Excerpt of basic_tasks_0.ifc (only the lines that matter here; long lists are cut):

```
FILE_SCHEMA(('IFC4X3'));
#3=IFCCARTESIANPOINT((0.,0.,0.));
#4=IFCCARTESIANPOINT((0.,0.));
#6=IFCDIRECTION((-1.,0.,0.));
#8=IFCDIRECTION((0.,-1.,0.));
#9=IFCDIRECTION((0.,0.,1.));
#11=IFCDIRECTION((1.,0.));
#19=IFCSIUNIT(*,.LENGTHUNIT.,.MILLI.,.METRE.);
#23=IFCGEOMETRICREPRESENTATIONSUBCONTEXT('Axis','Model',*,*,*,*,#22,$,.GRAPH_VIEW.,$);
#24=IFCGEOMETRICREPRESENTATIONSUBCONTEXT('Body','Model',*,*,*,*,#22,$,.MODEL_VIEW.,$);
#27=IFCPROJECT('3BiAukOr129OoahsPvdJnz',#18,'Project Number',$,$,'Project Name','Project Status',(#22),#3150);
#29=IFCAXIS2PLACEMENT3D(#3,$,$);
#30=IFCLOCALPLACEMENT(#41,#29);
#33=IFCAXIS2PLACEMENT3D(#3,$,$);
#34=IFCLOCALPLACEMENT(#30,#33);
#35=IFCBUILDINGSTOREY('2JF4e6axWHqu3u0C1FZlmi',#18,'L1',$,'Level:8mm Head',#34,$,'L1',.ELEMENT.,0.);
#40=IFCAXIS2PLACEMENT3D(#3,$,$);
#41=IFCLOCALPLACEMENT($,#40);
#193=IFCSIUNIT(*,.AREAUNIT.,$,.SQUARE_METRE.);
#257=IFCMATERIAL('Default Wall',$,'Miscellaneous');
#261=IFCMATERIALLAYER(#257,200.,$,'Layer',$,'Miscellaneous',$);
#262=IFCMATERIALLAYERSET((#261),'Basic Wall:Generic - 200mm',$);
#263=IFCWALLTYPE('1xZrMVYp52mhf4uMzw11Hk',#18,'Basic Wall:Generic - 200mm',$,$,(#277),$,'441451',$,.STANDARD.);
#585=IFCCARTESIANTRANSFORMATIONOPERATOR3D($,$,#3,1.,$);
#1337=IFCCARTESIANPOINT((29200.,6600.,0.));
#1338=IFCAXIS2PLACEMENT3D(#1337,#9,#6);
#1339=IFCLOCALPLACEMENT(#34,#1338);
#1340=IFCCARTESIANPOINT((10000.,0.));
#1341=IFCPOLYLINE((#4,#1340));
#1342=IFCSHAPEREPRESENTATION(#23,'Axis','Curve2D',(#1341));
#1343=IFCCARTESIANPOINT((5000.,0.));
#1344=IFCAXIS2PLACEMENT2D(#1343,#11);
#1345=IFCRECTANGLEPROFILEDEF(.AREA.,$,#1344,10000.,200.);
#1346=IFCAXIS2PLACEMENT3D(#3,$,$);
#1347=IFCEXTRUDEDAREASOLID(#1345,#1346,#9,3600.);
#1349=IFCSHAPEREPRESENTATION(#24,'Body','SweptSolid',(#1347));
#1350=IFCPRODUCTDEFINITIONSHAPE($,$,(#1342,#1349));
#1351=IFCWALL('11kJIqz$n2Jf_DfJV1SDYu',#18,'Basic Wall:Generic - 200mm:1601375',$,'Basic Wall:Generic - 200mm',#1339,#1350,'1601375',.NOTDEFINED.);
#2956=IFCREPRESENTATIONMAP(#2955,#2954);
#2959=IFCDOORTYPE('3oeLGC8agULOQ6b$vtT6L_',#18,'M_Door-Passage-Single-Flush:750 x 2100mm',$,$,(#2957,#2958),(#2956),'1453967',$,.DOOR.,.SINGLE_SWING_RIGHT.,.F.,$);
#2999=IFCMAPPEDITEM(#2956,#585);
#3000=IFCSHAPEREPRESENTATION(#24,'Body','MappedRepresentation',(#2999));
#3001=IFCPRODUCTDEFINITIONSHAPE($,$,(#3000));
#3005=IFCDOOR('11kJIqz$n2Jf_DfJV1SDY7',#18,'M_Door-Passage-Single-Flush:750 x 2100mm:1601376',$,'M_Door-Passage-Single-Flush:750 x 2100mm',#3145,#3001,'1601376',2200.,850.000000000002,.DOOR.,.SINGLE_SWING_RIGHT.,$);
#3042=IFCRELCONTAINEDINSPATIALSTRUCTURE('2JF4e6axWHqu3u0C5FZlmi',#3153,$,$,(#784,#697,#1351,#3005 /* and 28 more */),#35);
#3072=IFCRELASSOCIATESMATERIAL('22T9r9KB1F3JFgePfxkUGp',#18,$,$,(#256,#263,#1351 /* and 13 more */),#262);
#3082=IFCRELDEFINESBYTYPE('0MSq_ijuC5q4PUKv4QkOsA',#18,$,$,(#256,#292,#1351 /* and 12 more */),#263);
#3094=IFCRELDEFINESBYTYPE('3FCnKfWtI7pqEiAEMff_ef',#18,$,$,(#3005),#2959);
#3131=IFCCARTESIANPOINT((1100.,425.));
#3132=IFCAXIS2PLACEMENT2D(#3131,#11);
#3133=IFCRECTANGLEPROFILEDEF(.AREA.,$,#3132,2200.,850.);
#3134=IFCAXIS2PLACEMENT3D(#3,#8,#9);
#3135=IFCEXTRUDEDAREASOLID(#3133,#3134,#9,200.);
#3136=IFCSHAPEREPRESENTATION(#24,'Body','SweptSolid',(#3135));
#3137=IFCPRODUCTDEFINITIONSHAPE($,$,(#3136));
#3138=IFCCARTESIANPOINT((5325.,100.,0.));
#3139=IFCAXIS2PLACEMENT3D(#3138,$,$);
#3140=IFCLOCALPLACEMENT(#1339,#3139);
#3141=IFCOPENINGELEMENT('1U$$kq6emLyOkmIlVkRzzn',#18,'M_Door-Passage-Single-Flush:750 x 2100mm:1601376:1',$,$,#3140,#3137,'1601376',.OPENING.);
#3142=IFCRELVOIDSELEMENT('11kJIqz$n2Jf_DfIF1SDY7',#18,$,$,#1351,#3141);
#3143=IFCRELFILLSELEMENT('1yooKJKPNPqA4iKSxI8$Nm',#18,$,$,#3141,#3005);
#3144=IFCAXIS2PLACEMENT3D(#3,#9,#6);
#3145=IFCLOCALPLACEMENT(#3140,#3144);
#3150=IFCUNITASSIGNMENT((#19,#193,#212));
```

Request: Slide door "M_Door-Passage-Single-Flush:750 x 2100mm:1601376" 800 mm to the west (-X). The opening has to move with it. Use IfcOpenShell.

```python
import ifcopenshell
import ifcopenshell.api.geometry
import ifcopenshell.util.placement
import ifcopenshell.util.unit

model = ifcopenshell.open("basic_tasks_0.ifc")
unit_scale = ifcopenshell.util.unit.calculate_unit_scale(model)

door = model.by_id(3005)
opening = door.FillsVoids[0].RelatingOpeningElement
wall = opening.VoidsElements[0].RelatingBuildingElement

wall_matrix = ifcopenshell.util.placement.get_local_placement(wall.ObjectPlacement)
shift = wall_matrix[:3, 0] * 0.8 / unit_scale
before = ifcopenshell.util.placement.get_local_placement(door.ObjectPlacement)[:3, 3].copy()

# The door is placed relative to its opening, so it follows when the opening moves.
matrix = ifcopenshell.util.placement.get_local_placement(opening.ObjectPlacement)
matrix[:3, 3] += shift
ifcopenshell.api.geometry.edit_object_placement(
    model, product=opening, matrix=matrix, is_si=False, should_transform_children=True
)

after = ifcopenshell.util.placement.get_local_placement(door.ObjectPlacement)[:3, 3]
print("door moved by", (after - before).round(3) + 0.0)

model.write("basic_tasks_0_edited.ifc")
```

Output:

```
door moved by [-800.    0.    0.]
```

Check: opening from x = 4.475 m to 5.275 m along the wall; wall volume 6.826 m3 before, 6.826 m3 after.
